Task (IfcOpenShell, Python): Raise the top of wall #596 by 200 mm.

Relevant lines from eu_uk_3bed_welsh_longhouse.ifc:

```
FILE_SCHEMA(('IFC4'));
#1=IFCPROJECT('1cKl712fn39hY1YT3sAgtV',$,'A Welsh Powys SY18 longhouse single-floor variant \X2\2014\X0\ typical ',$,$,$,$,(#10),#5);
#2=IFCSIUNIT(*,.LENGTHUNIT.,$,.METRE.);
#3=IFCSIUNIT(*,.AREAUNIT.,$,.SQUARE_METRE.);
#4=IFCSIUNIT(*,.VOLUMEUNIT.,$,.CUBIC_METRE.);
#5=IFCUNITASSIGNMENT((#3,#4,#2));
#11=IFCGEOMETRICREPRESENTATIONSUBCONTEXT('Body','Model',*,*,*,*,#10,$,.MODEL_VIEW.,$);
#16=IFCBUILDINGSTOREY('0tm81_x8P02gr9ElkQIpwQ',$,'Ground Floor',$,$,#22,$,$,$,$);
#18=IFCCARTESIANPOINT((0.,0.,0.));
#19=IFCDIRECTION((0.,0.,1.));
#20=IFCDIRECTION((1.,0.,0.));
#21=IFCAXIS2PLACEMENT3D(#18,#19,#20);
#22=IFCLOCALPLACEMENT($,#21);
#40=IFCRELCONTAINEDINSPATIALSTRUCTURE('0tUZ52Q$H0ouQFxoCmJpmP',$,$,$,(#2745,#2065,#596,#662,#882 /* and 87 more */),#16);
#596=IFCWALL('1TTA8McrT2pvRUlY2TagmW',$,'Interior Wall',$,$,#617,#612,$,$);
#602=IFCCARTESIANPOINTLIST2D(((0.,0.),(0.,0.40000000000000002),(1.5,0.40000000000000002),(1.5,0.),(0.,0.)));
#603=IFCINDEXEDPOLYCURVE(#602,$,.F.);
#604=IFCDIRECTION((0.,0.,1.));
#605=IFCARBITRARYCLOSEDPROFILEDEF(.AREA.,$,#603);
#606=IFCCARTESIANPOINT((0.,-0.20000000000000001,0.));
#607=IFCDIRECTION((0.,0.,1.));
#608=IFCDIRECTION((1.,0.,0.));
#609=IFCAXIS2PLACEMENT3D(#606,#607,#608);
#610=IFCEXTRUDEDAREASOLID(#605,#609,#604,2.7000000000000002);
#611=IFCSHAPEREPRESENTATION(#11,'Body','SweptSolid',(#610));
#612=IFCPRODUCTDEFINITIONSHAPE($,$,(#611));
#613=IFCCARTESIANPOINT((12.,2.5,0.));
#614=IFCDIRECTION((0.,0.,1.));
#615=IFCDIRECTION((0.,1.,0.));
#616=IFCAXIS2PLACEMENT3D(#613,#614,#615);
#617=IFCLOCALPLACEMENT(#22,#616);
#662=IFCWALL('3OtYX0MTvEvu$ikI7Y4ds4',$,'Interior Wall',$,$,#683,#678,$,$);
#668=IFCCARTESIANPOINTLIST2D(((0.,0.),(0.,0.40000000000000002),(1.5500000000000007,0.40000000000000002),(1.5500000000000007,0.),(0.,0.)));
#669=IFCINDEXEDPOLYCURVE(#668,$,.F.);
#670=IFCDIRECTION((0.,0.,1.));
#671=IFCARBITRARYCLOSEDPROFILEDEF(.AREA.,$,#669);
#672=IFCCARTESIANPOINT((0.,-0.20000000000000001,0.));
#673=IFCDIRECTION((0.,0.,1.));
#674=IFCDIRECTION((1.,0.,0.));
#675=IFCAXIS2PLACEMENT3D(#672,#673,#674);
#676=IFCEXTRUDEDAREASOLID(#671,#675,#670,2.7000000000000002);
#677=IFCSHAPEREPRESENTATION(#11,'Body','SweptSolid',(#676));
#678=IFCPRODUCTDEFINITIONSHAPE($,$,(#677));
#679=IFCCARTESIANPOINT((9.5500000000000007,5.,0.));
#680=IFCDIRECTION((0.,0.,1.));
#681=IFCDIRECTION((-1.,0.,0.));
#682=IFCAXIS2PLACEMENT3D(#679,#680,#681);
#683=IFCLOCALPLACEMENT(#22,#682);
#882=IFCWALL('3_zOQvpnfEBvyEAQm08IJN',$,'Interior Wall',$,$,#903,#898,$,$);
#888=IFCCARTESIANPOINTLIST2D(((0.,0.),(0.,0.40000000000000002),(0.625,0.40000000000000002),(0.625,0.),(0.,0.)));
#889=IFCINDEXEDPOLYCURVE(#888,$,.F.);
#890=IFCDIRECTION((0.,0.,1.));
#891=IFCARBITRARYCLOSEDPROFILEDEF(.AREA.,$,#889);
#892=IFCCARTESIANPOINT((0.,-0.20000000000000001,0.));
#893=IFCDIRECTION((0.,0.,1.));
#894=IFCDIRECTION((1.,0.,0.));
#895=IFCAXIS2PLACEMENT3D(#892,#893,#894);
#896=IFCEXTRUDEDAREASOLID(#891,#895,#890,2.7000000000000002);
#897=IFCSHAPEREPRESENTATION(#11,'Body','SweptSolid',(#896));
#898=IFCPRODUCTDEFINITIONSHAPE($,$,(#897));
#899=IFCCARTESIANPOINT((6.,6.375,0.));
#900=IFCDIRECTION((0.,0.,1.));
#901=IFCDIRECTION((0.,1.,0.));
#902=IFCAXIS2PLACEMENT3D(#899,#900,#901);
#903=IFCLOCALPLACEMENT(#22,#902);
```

```python
import ifcopenshell
import ifcopenshell.geom
import ifcopenshell.util.representation
import ifcopenshell.util.shape
import ifcopenshell.util.unit

model = ifcopenshell.open("eu_uk_3bed_welsh_longhouse.ifc")
unit_scale = ifcopenshell.util.unit.calculate_unit_scale(model)
settings = ifcopenshell.geom.settings()


def volume(element):
    """Net volume in cubic metres, openings subtracted."""
    shape = ifcopenshell.geom.create_shape(settings, element)
    return ifcopenshell.util.shape.get_volume(shape.geometry)


wall = model.by_guid("1TTA8McrT2pvRUlY2TagmW")
before = volume(wall)

body = ifcopenshell.util.representation.get_representation(wall, "Model", "Body")
solid = body.Items[0]
old_height = solid.Depth
solid.Depth += 0.2 / unit_scale
after = volume(wall)

print(f"height {old_height:g} -> {solid.Depth:g}, volume {before:.3f} -> {after:.3f} m3")

model.write("eu_uk_3bed_welsh_longhouse_edited.ifc")
```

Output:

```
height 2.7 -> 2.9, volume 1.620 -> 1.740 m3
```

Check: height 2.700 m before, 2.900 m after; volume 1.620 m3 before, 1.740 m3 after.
